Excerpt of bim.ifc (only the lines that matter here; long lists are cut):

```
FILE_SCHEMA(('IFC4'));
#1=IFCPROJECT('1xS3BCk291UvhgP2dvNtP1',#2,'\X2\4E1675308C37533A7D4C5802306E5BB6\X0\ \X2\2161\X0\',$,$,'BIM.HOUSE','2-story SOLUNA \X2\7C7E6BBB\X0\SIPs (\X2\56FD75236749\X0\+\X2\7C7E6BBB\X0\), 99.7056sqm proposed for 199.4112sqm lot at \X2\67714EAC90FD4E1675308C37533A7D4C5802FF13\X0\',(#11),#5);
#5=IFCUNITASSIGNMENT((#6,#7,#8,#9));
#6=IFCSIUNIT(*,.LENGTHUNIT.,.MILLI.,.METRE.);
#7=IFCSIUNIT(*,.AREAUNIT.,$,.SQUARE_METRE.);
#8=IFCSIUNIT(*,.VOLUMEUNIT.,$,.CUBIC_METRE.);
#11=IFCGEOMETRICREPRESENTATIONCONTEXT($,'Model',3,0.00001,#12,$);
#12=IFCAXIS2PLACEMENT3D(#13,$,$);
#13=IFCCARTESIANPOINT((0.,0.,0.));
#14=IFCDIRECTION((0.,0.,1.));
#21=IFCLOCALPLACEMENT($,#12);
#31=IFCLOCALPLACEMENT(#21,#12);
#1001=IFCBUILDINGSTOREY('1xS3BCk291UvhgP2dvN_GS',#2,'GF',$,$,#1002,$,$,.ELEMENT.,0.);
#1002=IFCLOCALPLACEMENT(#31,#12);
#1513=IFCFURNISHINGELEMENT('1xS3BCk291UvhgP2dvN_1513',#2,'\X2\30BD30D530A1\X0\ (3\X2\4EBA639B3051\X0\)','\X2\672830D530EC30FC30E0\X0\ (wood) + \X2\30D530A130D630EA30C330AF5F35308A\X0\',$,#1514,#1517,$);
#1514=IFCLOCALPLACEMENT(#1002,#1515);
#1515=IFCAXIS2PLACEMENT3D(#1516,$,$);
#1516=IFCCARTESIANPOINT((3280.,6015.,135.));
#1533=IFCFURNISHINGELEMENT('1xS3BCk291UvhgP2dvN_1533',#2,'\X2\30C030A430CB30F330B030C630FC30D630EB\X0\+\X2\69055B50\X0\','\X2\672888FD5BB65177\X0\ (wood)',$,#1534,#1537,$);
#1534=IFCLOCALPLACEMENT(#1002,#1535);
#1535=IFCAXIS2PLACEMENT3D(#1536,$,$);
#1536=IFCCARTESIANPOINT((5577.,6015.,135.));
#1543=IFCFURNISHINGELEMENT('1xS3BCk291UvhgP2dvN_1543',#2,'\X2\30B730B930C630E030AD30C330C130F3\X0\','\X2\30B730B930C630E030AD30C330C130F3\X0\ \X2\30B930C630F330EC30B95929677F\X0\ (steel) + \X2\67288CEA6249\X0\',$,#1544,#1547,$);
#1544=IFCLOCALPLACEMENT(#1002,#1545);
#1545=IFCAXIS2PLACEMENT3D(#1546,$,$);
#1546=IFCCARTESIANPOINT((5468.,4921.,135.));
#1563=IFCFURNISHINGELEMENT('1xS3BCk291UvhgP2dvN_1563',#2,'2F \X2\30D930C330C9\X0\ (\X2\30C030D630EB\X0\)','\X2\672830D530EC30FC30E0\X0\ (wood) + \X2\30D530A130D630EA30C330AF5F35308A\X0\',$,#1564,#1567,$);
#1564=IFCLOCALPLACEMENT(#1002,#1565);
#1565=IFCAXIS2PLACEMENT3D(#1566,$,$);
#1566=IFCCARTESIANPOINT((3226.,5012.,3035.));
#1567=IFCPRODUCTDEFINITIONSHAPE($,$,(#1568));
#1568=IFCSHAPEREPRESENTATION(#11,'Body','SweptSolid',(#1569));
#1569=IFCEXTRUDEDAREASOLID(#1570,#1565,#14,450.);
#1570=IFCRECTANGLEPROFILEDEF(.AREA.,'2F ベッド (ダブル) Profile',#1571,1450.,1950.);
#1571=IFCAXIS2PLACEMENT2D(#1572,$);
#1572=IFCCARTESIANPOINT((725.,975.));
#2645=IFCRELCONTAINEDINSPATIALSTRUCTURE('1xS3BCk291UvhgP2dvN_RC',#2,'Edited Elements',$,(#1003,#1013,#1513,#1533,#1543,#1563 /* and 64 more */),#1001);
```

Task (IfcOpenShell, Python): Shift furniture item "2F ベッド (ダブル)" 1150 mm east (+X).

```python
import ifcopenshell
import ifcopenshell.api.geometry
import ifcopenshell.util.placement

model = ifcopenshell.open("bim.ifc")

item = model.by_guid("1xS3BCk291UvhgP2dvN_1563")
matrix = ifcopenshell.util.placement.get_local_placement(item.ObjectPlacement)
matrix[0, 3] += 1150.0
ifcopenshell.api.geometry.edit_object_placement(model, product=item, matrix=matrix, is_si=False)

print(ifcopenshell.util.placement.get_local_placement(item.ObjectPlacement).round(3) + 0.0)

model.write("bim-out.ifc")
```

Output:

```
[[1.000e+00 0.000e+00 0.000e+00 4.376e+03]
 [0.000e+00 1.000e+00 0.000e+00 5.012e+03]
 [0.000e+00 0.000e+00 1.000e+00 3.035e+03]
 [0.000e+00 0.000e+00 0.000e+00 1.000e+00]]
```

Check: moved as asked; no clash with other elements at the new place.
